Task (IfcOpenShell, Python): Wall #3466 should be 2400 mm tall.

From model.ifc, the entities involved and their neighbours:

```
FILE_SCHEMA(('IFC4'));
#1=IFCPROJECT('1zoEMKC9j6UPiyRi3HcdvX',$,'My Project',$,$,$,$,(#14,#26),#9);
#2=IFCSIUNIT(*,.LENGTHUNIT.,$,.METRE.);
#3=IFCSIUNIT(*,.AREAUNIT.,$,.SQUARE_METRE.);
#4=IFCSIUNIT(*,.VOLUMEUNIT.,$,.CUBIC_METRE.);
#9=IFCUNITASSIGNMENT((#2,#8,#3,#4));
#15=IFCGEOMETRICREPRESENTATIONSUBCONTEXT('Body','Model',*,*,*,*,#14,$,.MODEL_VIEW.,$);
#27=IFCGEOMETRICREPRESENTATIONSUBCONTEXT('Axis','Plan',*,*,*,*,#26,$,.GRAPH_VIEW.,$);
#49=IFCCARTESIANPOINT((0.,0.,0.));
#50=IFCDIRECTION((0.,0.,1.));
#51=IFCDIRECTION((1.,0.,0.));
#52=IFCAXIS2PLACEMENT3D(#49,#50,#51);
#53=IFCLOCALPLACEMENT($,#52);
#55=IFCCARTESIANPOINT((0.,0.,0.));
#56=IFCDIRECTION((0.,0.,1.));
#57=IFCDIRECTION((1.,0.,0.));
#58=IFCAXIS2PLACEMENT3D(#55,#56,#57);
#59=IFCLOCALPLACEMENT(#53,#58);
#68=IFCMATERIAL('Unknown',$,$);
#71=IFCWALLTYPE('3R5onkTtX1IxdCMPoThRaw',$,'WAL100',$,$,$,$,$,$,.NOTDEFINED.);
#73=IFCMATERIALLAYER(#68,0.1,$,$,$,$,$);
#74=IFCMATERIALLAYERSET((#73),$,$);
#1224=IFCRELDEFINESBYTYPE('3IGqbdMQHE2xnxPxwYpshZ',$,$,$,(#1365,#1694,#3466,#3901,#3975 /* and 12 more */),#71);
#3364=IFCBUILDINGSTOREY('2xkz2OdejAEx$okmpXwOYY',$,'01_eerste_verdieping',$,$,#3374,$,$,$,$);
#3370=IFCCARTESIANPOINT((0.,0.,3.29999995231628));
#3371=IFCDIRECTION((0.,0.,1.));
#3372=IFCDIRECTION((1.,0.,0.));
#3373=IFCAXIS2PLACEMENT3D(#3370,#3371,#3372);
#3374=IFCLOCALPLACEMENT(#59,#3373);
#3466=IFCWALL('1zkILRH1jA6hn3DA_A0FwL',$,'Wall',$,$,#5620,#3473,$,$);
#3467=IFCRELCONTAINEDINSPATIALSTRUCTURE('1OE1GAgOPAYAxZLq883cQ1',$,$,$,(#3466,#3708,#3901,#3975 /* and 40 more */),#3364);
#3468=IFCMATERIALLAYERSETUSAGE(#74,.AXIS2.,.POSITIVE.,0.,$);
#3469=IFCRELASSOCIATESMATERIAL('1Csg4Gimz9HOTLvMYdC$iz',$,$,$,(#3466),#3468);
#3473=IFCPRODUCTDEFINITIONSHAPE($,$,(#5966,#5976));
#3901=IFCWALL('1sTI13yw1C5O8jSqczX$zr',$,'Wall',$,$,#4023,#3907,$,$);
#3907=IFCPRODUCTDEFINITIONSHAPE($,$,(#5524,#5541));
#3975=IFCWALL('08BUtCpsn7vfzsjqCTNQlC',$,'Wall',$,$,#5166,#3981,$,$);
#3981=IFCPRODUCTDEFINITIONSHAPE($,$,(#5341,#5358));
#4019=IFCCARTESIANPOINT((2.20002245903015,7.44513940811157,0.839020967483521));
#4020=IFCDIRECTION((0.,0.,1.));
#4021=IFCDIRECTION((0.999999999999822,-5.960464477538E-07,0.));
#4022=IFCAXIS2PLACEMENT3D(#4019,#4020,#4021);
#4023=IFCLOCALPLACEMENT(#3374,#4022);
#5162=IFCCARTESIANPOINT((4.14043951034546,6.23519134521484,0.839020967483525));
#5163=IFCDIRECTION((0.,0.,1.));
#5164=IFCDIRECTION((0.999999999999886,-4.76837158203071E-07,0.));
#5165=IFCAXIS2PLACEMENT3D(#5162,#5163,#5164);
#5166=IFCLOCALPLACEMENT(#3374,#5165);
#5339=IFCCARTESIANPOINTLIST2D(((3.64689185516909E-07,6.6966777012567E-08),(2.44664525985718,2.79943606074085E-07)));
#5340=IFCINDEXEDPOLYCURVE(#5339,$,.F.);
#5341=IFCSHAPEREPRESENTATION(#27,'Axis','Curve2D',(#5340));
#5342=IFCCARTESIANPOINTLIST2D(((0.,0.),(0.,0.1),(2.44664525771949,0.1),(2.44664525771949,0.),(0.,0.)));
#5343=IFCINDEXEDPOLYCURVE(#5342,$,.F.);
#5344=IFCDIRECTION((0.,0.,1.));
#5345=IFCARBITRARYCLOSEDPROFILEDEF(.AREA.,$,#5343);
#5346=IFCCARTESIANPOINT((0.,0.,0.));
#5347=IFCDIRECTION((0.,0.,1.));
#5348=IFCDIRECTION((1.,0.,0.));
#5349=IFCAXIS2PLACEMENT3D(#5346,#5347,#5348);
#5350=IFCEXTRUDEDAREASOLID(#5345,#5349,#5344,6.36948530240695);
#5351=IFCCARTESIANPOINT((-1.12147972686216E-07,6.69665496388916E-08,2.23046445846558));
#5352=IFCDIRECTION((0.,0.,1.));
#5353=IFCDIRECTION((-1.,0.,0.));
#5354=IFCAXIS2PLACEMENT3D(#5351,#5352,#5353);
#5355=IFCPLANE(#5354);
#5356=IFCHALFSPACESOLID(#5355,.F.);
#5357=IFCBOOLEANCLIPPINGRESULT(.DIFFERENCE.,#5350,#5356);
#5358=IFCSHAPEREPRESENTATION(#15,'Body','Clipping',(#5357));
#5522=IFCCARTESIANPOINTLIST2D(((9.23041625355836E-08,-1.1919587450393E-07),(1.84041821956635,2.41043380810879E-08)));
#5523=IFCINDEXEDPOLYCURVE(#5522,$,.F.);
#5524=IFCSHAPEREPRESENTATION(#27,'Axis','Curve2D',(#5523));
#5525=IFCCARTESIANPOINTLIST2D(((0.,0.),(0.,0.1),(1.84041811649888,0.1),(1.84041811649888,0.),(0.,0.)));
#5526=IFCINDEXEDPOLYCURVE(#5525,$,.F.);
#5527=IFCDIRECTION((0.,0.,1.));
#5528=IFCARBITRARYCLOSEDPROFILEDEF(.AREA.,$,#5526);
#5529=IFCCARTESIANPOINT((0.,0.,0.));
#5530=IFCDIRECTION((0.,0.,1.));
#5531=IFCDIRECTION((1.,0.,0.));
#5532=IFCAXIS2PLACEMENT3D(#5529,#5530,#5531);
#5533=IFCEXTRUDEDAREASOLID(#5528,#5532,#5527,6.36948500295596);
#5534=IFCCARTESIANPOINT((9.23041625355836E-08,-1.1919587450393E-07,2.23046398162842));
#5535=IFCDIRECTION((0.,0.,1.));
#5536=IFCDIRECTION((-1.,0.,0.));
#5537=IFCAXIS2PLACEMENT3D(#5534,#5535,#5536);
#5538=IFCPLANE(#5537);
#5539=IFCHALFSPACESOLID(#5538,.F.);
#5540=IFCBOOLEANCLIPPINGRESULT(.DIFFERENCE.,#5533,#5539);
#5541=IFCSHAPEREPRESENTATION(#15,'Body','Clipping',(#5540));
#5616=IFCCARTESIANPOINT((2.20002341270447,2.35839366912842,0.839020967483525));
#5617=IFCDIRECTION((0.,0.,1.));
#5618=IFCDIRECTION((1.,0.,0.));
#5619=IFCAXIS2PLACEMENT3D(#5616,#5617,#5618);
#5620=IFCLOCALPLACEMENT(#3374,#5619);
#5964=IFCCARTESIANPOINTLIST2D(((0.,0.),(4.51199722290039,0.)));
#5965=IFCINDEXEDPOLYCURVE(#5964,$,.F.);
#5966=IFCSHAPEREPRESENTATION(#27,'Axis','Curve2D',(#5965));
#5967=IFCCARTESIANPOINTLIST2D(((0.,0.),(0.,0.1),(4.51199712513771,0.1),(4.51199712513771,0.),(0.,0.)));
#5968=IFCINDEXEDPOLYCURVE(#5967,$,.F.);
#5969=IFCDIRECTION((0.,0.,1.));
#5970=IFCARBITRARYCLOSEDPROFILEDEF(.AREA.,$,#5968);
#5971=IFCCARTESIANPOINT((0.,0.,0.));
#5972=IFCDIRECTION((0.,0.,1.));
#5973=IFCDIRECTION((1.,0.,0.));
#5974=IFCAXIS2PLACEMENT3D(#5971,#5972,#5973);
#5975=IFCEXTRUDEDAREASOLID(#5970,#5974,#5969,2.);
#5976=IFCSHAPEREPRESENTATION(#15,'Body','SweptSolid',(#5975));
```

```python
import ifcopenshell
import ifcopenshell.geom
import ifcopenshell.util.representation
import ifcopenshell.util.shape

model = ifcopenshell.open("model.ifc")
settings = ifcopenshell.geom.settings()


def volume(element):
    """Net volume in cubic metres, openings subtracted."""
    shape = ifcopenshell.geom.create_shape(settings, element)
    return ifcopenshell.util.shape.get_volume(shape.geometry)


wall = model.by_guid("1zkILRH1jA6hn3DA_A0FwL")
before = volume(wall)

body = ifcopenshell.util.representation.get_representation(wall, "Model", "Body")
solid = body.Items[0]
old_height = solid.Depth
solid.Depth = 2.4
after = volume(wall)

print(f"height {old_height:g} -> {solid.Depth:g}, volume {before:.3f} -> {after:.3f} m3")

model.write("model_updated.ifc")
```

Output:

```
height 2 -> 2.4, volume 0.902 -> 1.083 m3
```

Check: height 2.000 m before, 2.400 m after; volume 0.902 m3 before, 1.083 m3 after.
